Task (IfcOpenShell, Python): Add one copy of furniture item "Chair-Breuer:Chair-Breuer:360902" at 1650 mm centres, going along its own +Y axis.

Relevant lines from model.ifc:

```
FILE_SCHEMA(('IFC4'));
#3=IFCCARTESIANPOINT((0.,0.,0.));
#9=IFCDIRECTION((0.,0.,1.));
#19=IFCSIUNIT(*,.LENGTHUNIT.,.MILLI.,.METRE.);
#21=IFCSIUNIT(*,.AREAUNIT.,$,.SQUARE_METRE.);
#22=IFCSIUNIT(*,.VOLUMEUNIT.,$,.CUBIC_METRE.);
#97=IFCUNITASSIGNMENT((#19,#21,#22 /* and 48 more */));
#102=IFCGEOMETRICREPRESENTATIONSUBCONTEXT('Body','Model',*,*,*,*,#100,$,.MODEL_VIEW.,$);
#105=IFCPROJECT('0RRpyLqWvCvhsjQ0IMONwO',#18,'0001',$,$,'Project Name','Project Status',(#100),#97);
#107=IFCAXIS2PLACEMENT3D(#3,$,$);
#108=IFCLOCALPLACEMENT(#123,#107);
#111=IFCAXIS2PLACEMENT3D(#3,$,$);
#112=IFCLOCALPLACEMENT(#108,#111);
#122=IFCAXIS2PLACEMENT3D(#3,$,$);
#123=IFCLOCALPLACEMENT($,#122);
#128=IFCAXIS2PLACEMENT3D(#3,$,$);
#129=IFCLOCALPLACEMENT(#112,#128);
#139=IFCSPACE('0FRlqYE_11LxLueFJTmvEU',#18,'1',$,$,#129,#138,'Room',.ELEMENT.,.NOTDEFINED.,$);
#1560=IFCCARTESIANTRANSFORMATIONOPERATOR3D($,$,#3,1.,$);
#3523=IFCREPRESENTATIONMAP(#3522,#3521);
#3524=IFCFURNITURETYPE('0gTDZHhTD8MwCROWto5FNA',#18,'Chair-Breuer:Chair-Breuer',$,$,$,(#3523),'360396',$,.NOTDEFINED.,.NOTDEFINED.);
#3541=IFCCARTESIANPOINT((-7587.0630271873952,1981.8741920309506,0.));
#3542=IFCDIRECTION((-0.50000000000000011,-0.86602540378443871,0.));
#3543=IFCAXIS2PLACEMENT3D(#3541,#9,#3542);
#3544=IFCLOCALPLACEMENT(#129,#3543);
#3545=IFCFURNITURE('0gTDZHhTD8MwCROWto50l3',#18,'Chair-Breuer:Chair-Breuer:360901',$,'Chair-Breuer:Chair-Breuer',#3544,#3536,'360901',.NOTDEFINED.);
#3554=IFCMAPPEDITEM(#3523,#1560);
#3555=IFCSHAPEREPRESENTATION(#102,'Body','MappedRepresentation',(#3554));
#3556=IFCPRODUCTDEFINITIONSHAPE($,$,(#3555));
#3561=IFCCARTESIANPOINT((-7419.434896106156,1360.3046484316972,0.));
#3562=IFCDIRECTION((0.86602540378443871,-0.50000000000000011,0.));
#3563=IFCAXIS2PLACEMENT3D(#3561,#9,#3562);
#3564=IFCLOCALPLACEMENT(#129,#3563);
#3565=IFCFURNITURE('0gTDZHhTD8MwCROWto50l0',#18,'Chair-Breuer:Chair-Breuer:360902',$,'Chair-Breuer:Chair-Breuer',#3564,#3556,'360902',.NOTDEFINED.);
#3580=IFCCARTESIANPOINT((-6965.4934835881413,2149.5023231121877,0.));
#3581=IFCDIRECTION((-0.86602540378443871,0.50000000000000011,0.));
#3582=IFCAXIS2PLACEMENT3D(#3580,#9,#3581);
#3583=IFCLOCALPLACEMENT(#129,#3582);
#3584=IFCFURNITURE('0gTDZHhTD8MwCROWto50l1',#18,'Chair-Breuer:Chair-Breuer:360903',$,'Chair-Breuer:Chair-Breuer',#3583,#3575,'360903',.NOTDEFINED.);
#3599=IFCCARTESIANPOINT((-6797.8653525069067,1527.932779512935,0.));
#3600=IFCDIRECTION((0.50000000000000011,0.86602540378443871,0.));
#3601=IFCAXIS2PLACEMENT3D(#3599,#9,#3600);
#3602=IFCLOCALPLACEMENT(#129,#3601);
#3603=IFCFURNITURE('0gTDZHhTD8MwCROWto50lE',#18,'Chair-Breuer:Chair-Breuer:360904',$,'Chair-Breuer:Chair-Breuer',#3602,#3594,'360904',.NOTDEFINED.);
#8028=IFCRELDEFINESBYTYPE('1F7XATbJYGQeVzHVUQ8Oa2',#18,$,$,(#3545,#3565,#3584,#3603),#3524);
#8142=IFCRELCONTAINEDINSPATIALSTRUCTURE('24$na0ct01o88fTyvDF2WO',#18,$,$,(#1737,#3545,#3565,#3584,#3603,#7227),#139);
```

```python
import ifcopenshell
import ifcopenshell.api.geometry
import ifcopenshell.api.root
import ifcopenshell.util.element
import ifcopenshell.util.placement
import ifcopenshell.util.unit

model = ifcopenshell.open("model.ifc")
unit_scale = ifcopenshell.util.unit.calculate_unit_scale(model)


def reuse_history(source, copy):
    """copy_class also copies each property set's owner history, people and application; keep the originals."""
    for rel in copy.IsDefinedBy:
        if rel.is_a("IfcRelDefinesByProperties") and (history := rel.RelatingPropertyDefinition.OwnerHistory):
            rel.RelatingPropertyDefinition.OwnerHistory = source.OwnerHistory
            ifcopenshell.util.element.remove_deep2(model, history)


source = model.by_id(3565)
base = ifcopenshell.util.placement.get_local_placement(source.ObjectPlacement)
step = base[:3, 1] * 1.65 / unit_scale

for i in range(1, 2):
    copy = ifcopenshell.api.root.copy_class(model, product=source)
    copy.Representation = ifcopenshell.util.element.copy_deep(
        model, source.Representation, exclude=["IfcGeometricRepresentationContext", "IfcRepresentationMap"]
    )
    copy.Name = "Chair-Breuer:Chair-Breuer"
    copy.Tag = None
    reuse_history(source, copy)
    matrix = base.copy()
    matrix[:3, 3] += i * step
    print("added at", matrix[:3, 3].round(3) + 0.0)
    ifcopenshell.api.geometry.edit_object_placement(model, product=copy, matrix=matrix, is_si=False)

model.write("model_updated.ifc")
```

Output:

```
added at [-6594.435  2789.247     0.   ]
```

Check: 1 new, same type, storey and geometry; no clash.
